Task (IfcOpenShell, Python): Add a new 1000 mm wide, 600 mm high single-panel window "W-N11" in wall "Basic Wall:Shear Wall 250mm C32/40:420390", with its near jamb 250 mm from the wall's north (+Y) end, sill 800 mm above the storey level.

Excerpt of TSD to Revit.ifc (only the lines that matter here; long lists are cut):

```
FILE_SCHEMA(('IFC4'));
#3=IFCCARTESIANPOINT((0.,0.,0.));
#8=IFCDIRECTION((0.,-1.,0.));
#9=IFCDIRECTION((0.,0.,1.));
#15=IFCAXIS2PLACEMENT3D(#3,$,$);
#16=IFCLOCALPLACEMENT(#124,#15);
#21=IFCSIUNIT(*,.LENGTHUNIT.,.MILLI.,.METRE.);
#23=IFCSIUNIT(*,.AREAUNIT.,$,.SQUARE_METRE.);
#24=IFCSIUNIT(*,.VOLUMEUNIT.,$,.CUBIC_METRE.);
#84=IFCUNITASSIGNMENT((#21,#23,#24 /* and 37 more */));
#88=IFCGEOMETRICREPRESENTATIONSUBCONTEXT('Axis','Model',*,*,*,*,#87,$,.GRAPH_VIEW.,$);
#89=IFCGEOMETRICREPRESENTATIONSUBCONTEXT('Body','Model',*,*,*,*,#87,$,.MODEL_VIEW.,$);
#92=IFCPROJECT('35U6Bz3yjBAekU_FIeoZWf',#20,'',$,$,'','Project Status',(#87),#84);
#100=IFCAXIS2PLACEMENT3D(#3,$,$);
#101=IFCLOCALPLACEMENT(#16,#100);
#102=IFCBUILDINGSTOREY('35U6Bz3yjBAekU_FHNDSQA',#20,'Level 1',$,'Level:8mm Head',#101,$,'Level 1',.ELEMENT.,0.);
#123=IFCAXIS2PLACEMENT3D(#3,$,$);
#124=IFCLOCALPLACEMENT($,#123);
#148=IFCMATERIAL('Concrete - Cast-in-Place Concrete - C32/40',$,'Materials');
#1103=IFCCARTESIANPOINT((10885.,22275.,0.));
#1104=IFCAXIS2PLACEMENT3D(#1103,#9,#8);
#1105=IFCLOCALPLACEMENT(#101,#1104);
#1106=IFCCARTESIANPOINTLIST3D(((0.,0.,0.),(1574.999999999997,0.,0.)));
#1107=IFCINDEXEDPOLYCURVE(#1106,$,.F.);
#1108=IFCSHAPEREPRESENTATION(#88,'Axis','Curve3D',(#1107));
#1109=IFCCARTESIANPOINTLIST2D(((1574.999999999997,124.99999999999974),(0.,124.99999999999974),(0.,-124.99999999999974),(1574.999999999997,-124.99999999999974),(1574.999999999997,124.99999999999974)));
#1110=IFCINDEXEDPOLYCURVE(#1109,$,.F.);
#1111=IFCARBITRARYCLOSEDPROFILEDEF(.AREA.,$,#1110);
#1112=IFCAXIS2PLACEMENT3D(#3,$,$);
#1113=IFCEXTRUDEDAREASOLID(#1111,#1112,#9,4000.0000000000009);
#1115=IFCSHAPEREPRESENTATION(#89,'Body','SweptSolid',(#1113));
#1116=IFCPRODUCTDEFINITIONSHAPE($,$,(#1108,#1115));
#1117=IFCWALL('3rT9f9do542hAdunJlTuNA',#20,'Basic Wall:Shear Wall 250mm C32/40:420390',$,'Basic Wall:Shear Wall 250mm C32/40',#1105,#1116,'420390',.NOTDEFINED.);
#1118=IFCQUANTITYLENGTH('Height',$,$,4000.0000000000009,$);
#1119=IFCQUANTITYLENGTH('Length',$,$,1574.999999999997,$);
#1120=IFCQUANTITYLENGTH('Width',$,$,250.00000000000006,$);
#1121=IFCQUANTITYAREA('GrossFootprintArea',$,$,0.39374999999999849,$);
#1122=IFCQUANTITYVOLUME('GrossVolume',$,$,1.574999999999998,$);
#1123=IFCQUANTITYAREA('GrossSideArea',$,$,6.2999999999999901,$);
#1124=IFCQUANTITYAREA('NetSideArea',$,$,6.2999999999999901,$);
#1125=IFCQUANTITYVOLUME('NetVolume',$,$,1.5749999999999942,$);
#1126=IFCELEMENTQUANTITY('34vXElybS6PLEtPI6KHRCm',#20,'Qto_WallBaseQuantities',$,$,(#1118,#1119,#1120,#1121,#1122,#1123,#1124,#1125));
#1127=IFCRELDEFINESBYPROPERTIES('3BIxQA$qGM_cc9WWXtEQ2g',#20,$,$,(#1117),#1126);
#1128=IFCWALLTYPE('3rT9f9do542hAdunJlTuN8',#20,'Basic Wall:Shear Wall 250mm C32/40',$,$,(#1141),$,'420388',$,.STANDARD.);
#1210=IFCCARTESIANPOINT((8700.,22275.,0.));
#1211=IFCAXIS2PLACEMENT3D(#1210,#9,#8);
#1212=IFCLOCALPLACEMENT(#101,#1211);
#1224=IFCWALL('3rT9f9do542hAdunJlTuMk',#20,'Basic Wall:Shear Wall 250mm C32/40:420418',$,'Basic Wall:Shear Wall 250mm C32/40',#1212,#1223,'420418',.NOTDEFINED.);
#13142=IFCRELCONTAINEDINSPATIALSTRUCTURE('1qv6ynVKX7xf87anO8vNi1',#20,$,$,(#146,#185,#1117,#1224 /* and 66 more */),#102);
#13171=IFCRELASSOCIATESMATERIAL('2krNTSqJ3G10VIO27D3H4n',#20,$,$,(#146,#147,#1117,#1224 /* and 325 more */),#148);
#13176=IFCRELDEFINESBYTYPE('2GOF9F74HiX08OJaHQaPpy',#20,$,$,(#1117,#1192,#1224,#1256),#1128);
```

```python
import numpy as np
import ifcopenshell
import ifcopenshell.api.feature
import ifcopenshell.api.geometry
import ifcopenshell.api.pset
import ifcopenshell.api.root
import ifcopenshell.api.spatial
import ifcopenshell.geom
import ifcopenshell.util.element
import ifcopenshell.util.placement
import ifcopenshell.util.representation
import ifcopenshell.util.shape
import ifcopenshell.util.unit

model = ifcopenshell.open("TSD to Revit.ifc")
unit_scale = ifcopenshell.util.unit.calculate_unit_scale(model)
area_scale = ifcopenshell.util.unit.calculate_unit_scale(model, "AREAUNIT")
volume_scale = ifcopenshell.util.unit.calculate_unit_scale(model, "VOLUMEUNIT")
settings = ifcopenshell.geom.settings()


def volume(element):
    """Net volume in cubic metres, openings subtracted."""
    shape = ifcopenshell.geom.create_shape(settings, element)
    return ifcopenshell.util.shape.get_volume(shape.geometry)


wall = model.by_id(1117)
storey = ifcopenshell.util.element.get_container(wall, ifc_class="IfcBuildingStorey")
context = ifcopenshell.util.representation.get_context(model, "Model", "Body", "MODEL_VIEW")
before = volume(wall)

width, height, from_end, sill = 1, 0.6, 0.25, 0.8  # metres

# The wall runs along its own X axis, and the end named is its -X end.
wall_shape = ifcopenshell.geom.create_shape(settings, wall)
x, y, z = ifcopenshell.util.shape.get_vertices(wall_shape.geometry).T
start = x.min() + from_end
face, thickness = float(y.min()), float(y.max() - y.min())
wall_matrix = ifcopenshell.util.placement.get_local_placement(wall.ObjectPlacement)
level = ifcopenshell.util.placement.get_local_placement(storey.ObjectPlacement)[2, 3]


def in_wall(x, y):
    """Placement at x, y metres in the wall's axes, at sill height."""
    matrix = wall_matrix.copy()
    matrix[:, 3] = wall_matrix @ np.array([x / unit_scale, y / unit_scale, 0.0, 1.0])
    matrix[2, 3] = level + sill / unit_scale
    return matrix


# Opening: a box that overshoots both wall faces by 50 mm.
opening = ifcopenshell.api.root.create_entity(model, ifc_class="IfcOpeningElement", predefined_type="OPENING")
box = ifcopenshell.api.geometry.add_wall_representation(
    model, context=context, length=width, height=height, thickness=thickness + 0.1
)
ifcopenshell.api.geometry.assign_representation(model, product=opening, representation=box)
ifcopenshell.api.geometry.edit_object_placement(model, product=opening, matrix=in_wall(start, face - 0.05), is_si=False)
ifcopenshell.api.feature.add_feature(model, feature=opening, element=wall)

window = ifcopenshell.api.root.create_entity(model, ifc_class="IfcWindow", name="W-N11", predefined_type="WINDOW")
window.OverallWidth, window.OverallHeight = width / unit_scale, height / unit_scale
window.PartitioningType = "SINGLE_PANEL"
body = ifcopenshell.api.geometry.add_window_representation(
    model,
    context=context,
    overall_width=window.OverallWidth,
    overall_height=window.OverallHeight,
    partition_type="SINGLE_PANEL",
)
ifcopenshell.api.geometry.assign_representation(model, product=window, representation=body)
ifcopenshell.api.spatial.assign_container(model, products=[window], relating_structure=storey)
ifcopenshell.api.feature.add_filling(model, opening=opening, element=window)

# Centre the window in the wall's thickness.
ifcopenshell.api.geometry.edit_object_placement(model, product=window, matrix=in_wall(start, face), is_si=False)
window_shape = ifcopenshell.geom.create_shape(settings, window)
depth = ifcopenshell.util.shape.get_vertices(window_shape.geometry)[:, 1]
offset = face + thickness / 2 - (depth.min() + depth.max()) / 2
ifcopenshell.api.geometry.edit_object_placement(model, product=window, matrix=in_wall(start, offset), is_si=False)

after = volume(wall)

# Update the wall's stored quantities.
qto = model.by_id(ifcopenshell.util.element.get_pset(wall, "Qto_WallBaseQuantities", should_inherit=False)["id"])
ifcopenshell.api.pset.edit_qto(model, qto=qto, properties={
    "NetSideArea": after / thickness / area_scale,
    "NetVolume": after / volume_scale,
})

print(f"wall volume {before:.3f} -> {after:.3f} m3")

model.write("TSD to Revit_edited.ifc")
```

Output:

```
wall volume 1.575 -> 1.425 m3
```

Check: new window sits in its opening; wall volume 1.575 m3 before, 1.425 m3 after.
